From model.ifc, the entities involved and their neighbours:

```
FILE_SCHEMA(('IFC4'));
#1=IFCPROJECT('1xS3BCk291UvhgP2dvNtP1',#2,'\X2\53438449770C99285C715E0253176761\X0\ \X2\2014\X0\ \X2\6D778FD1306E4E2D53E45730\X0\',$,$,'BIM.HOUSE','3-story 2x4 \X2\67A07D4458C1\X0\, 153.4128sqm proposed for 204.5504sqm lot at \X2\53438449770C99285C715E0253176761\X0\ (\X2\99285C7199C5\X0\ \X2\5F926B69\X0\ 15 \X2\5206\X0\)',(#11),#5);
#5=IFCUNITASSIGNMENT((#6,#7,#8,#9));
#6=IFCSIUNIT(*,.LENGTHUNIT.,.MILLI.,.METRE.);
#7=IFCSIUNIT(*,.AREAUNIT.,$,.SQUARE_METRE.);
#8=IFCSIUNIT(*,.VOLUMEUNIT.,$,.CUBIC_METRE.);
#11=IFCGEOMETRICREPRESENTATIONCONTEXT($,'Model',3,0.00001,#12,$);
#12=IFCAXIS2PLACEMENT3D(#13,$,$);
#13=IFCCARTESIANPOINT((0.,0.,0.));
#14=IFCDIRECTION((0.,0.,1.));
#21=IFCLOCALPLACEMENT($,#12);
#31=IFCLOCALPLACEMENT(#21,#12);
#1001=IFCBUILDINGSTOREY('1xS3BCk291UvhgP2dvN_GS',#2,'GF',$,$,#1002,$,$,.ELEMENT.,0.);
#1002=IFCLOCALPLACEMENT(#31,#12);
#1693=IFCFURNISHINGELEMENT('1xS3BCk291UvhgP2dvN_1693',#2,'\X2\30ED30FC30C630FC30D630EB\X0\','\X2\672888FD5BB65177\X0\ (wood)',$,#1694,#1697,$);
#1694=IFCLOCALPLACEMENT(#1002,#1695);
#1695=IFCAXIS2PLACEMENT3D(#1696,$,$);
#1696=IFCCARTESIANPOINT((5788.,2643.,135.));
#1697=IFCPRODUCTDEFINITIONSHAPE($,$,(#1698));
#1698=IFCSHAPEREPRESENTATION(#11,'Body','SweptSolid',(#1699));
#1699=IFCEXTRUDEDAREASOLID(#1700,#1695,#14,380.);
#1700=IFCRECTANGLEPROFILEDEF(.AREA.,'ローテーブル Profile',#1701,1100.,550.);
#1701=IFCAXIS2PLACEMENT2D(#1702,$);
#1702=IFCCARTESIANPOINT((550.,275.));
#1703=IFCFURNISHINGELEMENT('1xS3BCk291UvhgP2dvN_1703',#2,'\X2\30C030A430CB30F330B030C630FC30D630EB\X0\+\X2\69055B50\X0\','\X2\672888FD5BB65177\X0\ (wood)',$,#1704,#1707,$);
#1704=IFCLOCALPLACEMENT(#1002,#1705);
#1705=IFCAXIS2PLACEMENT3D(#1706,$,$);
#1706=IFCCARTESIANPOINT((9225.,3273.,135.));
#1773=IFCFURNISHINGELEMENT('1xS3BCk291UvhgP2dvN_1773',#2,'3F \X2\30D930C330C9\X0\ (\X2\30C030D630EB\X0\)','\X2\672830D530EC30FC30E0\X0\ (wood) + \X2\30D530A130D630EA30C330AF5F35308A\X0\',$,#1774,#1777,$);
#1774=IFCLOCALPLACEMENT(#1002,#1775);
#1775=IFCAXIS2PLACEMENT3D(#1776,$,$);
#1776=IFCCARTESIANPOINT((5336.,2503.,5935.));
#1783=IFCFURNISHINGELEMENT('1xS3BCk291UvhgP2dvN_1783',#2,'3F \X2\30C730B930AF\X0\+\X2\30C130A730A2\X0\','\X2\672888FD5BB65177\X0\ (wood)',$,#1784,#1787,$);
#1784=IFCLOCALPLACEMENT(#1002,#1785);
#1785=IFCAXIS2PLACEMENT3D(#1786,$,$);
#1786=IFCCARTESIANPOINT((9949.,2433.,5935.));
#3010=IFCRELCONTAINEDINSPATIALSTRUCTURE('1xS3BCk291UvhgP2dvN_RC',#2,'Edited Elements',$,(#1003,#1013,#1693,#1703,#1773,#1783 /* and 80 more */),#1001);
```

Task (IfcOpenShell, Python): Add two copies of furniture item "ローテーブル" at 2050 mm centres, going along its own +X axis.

```python
import ifcopenshell
import ifcopenshell.api.geometry
import ifcopenshell.api.root
import ifcopenshell.util.element
import ifcopenshell.util.placement

model = ifcopenshell.open("model.ifc")


def reuse_history(source, copy):
    """copy_class also copies each property set's owner history, people and application; keep the originals."""
    for rel in copy.IsDefinedBy:
        if rel.is_a("IfcRelDefinesByProperties") and (history := rel.RelatingPropertyDefinition.OwnerHistory):
            rel.RelatingPropertyDefinition.OwnerHistory = source.OwnerHistory
            ifcopenshell.util.element.remove_deep2(model, history)


source = model.by_guid("1xS3BCk291UvhgP2dvN_1693")
base = ifcopenshell.util.placement.get_local_placement(source.ObjectPlacement)
step = base[:3, 0] * 2050.0

for i in range(1, 3):
    copy = ifcopenshell.api.root.copy_class(model, product=source)
    copy.Representation = ifcopenshell.util.element.copy_deep(
        model, source.Representation, exclude=["IfcGeometricRepresentationContext", "IfcRepresentationMap"]
    )
    reuse_history(source, copy)
    matrix = base.copy()
    matrix[:3, 3] += i * step
    print("added at", matrix[:3, 3].round(3) + 0.0)
    ifcopenshell.api.geometry.edit_object_placement(model, product=copy, matrix=matrix, is_si=False)

model.write("model-out.ifc")
```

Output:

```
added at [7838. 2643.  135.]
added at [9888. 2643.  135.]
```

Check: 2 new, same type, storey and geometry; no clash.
